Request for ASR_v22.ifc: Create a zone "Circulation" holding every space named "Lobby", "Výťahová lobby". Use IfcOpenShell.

First a look at what the model holds.

```python
import ifcopenshell

model = ifcopenshell.open("ASR_v22.ifc")
print(model.schema)
seen = {}
for space in model.by_type("IfcSpace"):
    seen[space.LongName] = seen.get(space.LongName, 0) + 1
for name, count in sorted(seen.items(), key=str):
    print(count, "x", name)
print("zones:", [z.Name for z in model.by_type("IfcZone")][:20])
```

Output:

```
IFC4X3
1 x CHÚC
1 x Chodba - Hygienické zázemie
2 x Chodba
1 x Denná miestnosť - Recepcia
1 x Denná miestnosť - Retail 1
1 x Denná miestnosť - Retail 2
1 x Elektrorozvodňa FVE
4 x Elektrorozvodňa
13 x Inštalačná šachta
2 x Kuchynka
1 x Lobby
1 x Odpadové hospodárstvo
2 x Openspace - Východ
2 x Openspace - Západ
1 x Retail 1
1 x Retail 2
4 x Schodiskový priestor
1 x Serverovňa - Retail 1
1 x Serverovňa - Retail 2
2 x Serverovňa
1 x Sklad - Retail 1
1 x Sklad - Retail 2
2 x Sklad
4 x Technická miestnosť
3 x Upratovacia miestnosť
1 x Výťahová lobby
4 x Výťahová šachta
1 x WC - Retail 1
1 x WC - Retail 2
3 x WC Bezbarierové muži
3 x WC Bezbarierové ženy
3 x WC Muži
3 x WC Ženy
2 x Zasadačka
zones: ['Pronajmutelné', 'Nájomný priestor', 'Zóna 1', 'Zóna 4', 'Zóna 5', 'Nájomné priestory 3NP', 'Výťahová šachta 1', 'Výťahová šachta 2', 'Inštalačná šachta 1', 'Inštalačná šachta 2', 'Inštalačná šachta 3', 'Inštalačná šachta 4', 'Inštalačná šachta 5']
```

```python
import ifcopenshell
import ifcopenshell.api.group
import ifcopenshell.api.root

model = ifcopenshell.open("ASR_v22.ifc")

names = {"Lobby", "Výťahová lobby"}
spaces = [s for s in model.by_type("IfcSpace") if s.LongName in names]

zone = ifcopenshell.api.root.create_entity(model, ifc_class="IfcZone", name="Circulation")
ifcopenshell.api.group.assign_group(model, products=spaces, group=zone)
print(len(spaces), "spaces in", zone.Name)

model.write("ASR_v22_updated.ifc")
```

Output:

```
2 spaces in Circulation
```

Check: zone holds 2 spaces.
